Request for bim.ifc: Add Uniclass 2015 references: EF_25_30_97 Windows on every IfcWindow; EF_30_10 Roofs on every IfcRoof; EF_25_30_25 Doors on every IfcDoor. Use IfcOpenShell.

First a look at what the model holds.

```python
import ifcopenshell

model = ifcopenshell.open("bim.ifc")
print(model.schema)
print("classifications:", [c.Name for c in model.by_type("IfcClassification")])
for ifc_class in ("IfcDoor", "IfcRoof", "IfcStair", "IfcWall", "IfcWindow"):
    print(ifc_class, len(model.by_type(ifc_class)))
```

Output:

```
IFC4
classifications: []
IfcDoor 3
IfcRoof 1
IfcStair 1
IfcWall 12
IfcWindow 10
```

```python
import ifcopenshell
import ifcopenshell.api.classification

model = ifcopenshell.open("bim.ifc")

system = ifcopenshell.api.classification.add_classification(model, classification="Uniclass 2015")

codes = {
    "IfcWindow": ("EF_25_30_97", "Windows"),
    "IfcRoof": ("EF_30_10", "Roofs"),
    "IfcDoor": ("EF_25_30_25", "Doors"),
}
for ifc_class, (code, name) in codes.items():
    products = model.by_type(ifc_class)
    ifcopenshell.api.classification.add_reference(
        model, products=products, classification=system, identification=code, name=name
    )
    print(code, len(products))

model.write("bim_v2.ifc")
```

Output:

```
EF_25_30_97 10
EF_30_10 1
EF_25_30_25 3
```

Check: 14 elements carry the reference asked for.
